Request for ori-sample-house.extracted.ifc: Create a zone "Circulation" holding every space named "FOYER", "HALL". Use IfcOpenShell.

First a look at what the model holds.

```python
import ifcopenshell

model = ifcopenshell.open("ori-sample-house.extracted.ifc")
print(model.schema)
seen = {}
for space in model.by_type("IfcSpace"):
    seen[space.Name] = seen.get(space.Name, 0) + 1
for name, count in sorted(seen.items(), key=str):
    print(count, "x", name)
print("zones:", [z.Name for z in model.by_type("IfcZone")][:20])
```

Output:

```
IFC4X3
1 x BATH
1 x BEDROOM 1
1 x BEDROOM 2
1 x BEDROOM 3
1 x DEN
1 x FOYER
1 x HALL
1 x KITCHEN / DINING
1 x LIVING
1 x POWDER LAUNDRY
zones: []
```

```python
import ifcopenshell
import ifcopenshell.api.group
import ifcopenshell.api.root

model = ifcopenshell.open("ori-sample-house.extracted.ifc")

names = {"FOYER", "HALL"}
spaces = [s for s in model.by_type("IfcSpace") if s.Name in names]

zone = ifcopenshell.api.root.create_entity(model, ifc_class="IfcZone", name="Circulation")
ifcopenshell.api.group.assign_group(model, products=spaces, group=zone)
print(len(spaces), "spaces in", zone.Name)

model.write("ori-sample-house.extracted_edited.ifc")
```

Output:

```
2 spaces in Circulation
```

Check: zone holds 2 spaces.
